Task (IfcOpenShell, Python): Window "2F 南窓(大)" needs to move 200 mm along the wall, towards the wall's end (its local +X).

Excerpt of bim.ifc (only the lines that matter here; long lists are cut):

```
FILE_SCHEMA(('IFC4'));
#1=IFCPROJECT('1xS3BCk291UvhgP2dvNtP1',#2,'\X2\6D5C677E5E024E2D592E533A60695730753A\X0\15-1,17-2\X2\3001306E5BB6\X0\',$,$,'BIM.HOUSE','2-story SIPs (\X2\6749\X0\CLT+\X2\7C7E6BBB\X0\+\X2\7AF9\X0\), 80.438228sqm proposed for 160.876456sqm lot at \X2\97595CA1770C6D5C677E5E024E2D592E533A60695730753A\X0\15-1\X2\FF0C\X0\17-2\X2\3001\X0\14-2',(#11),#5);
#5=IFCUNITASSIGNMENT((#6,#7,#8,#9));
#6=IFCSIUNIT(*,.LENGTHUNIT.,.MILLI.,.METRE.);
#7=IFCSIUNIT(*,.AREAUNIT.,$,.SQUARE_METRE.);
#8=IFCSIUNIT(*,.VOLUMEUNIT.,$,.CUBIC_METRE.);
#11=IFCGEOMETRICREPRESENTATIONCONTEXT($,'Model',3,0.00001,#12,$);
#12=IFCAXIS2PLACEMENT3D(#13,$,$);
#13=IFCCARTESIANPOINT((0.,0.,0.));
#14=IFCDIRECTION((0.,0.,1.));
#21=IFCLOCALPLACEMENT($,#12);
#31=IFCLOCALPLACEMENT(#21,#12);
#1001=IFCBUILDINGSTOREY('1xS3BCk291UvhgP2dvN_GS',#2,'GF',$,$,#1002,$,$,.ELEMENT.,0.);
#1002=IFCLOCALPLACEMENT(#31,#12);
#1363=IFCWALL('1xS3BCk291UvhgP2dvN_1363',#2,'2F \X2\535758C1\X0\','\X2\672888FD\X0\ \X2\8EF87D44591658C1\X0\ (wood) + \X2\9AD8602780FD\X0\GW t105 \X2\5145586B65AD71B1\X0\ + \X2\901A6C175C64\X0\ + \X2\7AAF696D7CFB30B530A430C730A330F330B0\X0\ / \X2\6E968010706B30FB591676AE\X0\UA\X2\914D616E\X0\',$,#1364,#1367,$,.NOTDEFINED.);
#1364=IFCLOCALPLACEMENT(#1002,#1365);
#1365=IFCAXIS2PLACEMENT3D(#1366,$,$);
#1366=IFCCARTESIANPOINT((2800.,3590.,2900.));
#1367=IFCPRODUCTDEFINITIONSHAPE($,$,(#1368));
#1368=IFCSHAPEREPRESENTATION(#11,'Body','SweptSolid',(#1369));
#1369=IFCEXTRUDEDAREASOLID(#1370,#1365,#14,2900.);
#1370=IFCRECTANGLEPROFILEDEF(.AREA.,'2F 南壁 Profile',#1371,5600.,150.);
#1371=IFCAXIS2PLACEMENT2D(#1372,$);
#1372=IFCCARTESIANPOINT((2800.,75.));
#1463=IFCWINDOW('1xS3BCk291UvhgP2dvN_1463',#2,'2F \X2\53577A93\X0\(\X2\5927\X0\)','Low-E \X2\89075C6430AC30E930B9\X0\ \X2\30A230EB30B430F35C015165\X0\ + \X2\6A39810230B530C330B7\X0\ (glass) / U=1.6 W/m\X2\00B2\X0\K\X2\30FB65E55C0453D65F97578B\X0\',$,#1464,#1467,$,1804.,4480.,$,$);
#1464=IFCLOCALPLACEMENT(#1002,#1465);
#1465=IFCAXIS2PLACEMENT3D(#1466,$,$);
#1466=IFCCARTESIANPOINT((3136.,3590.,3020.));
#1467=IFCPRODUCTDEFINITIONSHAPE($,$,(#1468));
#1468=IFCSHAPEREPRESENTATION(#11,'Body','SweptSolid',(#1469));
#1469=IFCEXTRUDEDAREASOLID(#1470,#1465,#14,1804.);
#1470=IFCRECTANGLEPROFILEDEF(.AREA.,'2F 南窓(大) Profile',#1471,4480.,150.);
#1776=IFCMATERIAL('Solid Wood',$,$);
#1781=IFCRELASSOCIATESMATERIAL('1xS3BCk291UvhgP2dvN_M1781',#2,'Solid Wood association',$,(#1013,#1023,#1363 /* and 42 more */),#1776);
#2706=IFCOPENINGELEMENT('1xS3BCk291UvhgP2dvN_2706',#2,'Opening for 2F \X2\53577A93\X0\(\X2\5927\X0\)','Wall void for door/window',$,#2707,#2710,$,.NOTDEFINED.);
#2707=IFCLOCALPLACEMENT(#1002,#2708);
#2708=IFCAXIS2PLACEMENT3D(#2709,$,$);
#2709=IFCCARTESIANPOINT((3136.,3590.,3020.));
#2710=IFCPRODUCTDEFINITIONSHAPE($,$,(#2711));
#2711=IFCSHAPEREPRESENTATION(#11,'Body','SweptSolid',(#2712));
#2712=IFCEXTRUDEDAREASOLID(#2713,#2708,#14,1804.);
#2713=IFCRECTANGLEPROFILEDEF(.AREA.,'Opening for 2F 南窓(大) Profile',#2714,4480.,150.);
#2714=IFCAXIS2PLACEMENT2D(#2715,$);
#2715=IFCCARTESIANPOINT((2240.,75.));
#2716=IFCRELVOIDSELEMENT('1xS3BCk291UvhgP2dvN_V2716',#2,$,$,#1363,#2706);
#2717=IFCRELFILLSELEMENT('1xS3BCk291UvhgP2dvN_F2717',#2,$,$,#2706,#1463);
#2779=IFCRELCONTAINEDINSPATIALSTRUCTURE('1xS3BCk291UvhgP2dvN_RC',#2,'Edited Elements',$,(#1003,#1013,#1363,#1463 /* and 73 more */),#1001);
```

```python
import ifcopenshell
import ifcopenshell.api.geometry
import ifcopenshell.util.placement
import ifcopenshell.util.unit

model = ifcopenshell.open("bim.ifc")
unit_scale = ifcopenshell.util.unit.calculate_unit_scale(model)

window = model.by_guid("1xS3BCk291UvhgP2dvN_1463")
opening = window.FillsVoids[0].RelatingOpeningElement
wall = opening.VoidsElements[0].RelatingBuildingElement

wall_matrix = ifcopenshell.util.placement.get_local_placement(wall.ObjectPlacement)
shift = wall_matrix[:3, 0] * 0.2 / unit_scale
before = ifcopenshell.util.placement.get_local_placement(window.ObjectPlacement)[:3, 3].copy()

# The window is not placed relative to its opening, so move both.
for product in (opening, window):
    matrix = ifcopenshell.util.placement.get_local_placement(product.ObjectPlacement)
    matrix[:3, 3] += shift
    ifcopenshell.api.geometry.edit_object_placement(model, product=product, matrix=matrix, is_si=False)

after = ifcopenshell.util.placement.get_local_placement(window.ObjectPlacement)[:3, 3]
print("window moved by", (after - before).round(3) + 0.0)

model.write("bim_rev.ifc")
```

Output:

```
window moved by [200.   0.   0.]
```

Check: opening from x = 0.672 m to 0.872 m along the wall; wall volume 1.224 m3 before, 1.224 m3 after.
